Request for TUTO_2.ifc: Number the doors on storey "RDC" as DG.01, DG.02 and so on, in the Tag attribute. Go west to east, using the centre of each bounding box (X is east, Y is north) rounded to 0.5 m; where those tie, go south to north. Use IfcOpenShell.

First a look at what the model holds.

```python
import ifcopenshell
import ifcopenshell.util.element
import ifcopenshell.util.placement

model = ifcopenshell.open("TUTO_2.ifc")
print(model.schema)
storey = next(s for s in model.by_type("IfcBuildingStorey") if s.Name == "RDC")
doors = [e for e in ifcopenshell.util.element.get_decomposition(storey) if e.is_a("IfcDoor")]
for e in sorted(doors, key=lambda e: e.id()):
    origin = ifcopenshell.util.placement.get_local_placement(e.ObjectPlacement)[:3, 3]
    print(e.id(), e.Tag, e.Name, origin.round(2) + 0.0, sep=" | ")
```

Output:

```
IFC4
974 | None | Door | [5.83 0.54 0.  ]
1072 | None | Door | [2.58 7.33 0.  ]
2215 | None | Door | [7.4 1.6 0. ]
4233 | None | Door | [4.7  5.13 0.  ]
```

```python
import ifcopenshell
import ifcopenshell.geom
import ifcopenshell.util.element
import ifcopenshell.util.shape

model = ifcopenshell.open("TUTO_2.ifc")
settings = ifcopenshell.geom.settings()
settings.set("use-world-coords", True)


def centre(element):
    shape = ifcopenshell.geom.create_shape(settings, element)
    return ifcopenshell.util.shape.get_bbox_centroid(shape.geometry)


storey = next(s for s in model.by_type("IfcBuildingStorey") if s.Name == "RDC")
doors = [e for e in ifcopenshell.util.element.get_decomposition(storey) if e.is_a("IfcDoor")]

# Insertion points can sit at a corner or the storey origin, so sort by the geometry (in metres).
centres = {e: centre(e) for e in doors}
doors.sort(key=lambda e: (round(centres[e][0] / 0.5), centres[e][1]))

for i, e in enumerate(doors, start=1):
    number = f"DG.{i:02d}"
    e.Tag = number
    print(e.id(), number)

model.write("TUTO_2_updated.ifc")
```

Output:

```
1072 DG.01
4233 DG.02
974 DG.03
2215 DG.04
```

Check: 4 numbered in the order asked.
